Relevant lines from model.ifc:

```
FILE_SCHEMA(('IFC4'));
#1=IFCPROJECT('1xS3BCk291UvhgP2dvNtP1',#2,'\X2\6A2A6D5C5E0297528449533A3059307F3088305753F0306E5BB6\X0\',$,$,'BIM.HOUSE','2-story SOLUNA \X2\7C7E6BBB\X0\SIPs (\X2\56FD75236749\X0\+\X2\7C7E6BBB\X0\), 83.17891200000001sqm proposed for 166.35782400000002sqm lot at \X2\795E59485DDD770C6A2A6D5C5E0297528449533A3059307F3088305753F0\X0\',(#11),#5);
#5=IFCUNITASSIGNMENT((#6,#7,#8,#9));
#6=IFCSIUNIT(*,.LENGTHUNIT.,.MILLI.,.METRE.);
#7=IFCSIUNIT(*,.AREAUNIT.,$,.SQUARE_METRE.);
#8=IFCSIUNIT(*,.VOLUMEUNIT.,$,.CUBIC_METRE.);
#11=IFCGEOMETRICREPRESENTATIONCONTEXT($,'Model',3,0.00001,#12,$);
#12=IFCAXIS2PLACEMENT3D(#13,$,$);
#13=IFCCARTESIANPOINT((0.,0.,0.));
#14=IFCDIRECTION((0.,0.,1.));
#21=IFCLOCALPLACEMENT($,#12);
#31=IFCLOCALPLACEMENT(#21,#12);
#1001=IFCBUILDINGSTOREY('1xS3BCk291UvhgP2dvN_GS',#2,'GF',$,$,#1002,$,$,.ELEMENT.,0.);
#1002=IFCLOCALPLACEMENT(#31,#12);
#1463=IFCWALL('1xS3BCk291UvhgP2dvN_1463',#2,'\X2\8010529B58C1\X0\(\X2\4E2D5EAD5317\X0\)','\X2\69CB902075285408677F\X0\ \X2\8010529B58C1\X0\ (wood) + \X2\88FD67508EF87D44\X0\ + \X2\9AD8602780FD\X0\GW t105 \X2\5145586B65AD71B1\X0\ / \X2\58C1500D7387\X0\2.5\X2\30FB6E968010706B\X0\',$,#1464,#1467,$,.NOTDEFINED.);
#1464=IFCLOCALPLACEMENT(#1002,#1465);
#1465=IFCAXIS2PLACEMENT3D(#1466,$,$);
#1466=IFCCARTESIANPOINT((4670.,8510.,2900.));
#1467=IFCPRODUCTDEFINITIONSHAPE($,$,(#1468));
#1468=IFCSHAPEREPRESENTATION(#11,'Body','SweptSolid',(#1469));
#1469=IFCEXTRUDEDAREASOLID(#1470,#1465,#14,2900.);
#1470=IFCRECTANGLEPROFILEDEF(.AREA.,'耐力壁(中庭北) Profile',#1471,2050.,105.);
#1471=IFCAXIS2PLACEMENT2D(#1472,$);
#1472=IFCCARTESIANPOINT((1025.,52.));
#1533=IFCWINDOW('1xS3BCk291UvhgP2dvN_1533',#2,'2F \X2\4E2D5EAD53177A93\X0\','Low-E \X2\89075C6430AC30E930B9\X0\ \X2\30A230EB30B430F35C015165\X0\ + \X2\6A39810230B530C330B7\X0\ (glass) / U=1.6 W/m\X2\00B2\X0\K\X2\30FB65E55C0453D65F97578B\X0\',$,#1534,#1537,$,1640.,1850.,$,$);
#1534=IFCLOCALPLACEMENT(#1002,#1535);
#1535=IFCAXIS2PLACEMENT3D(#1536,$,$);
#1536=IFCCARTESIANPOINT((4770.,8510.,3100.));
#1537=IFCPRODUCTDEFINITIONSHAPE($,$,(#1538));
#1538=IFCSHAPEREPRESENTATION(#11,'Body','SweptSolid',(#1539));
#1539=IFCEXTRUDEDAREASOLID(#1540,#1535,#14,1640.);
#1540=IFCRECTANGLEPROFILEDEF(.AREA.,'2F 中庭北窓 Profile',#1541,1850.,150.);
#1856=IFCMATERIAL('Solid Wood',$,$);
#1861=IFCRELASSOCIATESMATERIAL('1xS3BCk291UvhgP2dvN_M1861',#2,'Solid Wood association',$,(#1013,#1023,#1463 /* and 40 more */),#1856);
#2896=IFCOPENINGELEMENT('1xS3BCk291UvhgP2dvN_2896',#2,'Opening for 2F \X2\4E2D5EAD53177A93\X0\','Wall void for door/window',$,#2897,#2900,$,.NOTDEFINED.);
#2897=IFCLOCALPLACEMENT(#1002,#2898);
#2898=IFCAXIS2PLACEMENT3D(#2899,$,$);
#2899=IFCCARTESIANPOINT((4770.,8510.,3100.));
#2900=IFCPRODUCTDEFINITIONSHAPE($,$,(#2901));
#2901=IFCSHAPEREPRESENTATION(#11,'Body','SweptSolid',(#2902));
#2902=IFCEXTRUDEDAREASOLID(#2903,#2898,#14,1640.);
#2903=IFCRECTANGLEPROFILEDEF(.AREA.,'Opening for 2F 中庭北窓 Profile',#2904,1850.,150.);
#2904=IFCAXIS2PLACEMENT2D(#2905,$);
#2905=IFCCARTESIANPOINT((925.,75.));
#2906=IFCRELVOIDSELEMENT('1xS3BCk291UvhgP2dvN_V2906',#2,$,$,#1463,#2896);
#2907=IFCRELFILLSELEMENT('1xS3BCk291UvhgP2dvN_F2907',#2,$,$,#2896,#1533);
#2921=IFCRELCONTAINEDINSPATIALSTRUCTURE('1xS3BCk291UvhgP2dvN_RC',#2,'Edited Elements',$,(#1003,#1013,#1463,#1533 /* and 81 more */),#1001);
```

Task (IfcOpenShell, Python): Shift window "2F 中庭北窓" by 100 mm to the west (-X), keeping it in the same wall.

```python
import ifcopenshell
import ifcopenshell.api.geometry
import ifcopenshell.util.placement
import ifcopenshell.util.unit

model = ifcopenshell.open("model.ifc")
unit_scale = ifcopenshell.util.unit.calculate_unit_scale(model)

window = model.by_id(1533)
opening = window.FillsVoids[0].RelatingOpeningElement
wall = opening.VoidsElements[0].RelatingBuildingElement

wall_matrix = ifcopenshell.util.placement.get_local_placement(wall.ObjectPlacement)
shift = wall_matrix[:3, 0] * -0.1 / unit_scale
before = ifcopenshell.util.placement.get_local_placement(window.ObjectPlacement)[:3, 3].copy()

# The window is not placed relative to its opening, so move both.
for product in (opening, window):
    matrix = ifcopenshell.util.placement.get_local_placement(product.ObjectPlacement)
    matrix[:3, 3] += shift
    ifcopenshell.api.geometry.edit_object_placement(model, product=product, matrix=matrix, is_si=False)

after = ifcopenshell.util.placement.get_local_placement(window.ObjectPlacement)[:3, 3]
print("window moved by", (after - before).round(3) + 0.0)

model.write("model_edited.ifc")
```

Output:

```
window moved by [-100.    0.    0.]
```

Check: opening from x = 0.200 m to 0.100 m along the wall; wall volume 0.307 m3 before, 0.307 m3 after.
